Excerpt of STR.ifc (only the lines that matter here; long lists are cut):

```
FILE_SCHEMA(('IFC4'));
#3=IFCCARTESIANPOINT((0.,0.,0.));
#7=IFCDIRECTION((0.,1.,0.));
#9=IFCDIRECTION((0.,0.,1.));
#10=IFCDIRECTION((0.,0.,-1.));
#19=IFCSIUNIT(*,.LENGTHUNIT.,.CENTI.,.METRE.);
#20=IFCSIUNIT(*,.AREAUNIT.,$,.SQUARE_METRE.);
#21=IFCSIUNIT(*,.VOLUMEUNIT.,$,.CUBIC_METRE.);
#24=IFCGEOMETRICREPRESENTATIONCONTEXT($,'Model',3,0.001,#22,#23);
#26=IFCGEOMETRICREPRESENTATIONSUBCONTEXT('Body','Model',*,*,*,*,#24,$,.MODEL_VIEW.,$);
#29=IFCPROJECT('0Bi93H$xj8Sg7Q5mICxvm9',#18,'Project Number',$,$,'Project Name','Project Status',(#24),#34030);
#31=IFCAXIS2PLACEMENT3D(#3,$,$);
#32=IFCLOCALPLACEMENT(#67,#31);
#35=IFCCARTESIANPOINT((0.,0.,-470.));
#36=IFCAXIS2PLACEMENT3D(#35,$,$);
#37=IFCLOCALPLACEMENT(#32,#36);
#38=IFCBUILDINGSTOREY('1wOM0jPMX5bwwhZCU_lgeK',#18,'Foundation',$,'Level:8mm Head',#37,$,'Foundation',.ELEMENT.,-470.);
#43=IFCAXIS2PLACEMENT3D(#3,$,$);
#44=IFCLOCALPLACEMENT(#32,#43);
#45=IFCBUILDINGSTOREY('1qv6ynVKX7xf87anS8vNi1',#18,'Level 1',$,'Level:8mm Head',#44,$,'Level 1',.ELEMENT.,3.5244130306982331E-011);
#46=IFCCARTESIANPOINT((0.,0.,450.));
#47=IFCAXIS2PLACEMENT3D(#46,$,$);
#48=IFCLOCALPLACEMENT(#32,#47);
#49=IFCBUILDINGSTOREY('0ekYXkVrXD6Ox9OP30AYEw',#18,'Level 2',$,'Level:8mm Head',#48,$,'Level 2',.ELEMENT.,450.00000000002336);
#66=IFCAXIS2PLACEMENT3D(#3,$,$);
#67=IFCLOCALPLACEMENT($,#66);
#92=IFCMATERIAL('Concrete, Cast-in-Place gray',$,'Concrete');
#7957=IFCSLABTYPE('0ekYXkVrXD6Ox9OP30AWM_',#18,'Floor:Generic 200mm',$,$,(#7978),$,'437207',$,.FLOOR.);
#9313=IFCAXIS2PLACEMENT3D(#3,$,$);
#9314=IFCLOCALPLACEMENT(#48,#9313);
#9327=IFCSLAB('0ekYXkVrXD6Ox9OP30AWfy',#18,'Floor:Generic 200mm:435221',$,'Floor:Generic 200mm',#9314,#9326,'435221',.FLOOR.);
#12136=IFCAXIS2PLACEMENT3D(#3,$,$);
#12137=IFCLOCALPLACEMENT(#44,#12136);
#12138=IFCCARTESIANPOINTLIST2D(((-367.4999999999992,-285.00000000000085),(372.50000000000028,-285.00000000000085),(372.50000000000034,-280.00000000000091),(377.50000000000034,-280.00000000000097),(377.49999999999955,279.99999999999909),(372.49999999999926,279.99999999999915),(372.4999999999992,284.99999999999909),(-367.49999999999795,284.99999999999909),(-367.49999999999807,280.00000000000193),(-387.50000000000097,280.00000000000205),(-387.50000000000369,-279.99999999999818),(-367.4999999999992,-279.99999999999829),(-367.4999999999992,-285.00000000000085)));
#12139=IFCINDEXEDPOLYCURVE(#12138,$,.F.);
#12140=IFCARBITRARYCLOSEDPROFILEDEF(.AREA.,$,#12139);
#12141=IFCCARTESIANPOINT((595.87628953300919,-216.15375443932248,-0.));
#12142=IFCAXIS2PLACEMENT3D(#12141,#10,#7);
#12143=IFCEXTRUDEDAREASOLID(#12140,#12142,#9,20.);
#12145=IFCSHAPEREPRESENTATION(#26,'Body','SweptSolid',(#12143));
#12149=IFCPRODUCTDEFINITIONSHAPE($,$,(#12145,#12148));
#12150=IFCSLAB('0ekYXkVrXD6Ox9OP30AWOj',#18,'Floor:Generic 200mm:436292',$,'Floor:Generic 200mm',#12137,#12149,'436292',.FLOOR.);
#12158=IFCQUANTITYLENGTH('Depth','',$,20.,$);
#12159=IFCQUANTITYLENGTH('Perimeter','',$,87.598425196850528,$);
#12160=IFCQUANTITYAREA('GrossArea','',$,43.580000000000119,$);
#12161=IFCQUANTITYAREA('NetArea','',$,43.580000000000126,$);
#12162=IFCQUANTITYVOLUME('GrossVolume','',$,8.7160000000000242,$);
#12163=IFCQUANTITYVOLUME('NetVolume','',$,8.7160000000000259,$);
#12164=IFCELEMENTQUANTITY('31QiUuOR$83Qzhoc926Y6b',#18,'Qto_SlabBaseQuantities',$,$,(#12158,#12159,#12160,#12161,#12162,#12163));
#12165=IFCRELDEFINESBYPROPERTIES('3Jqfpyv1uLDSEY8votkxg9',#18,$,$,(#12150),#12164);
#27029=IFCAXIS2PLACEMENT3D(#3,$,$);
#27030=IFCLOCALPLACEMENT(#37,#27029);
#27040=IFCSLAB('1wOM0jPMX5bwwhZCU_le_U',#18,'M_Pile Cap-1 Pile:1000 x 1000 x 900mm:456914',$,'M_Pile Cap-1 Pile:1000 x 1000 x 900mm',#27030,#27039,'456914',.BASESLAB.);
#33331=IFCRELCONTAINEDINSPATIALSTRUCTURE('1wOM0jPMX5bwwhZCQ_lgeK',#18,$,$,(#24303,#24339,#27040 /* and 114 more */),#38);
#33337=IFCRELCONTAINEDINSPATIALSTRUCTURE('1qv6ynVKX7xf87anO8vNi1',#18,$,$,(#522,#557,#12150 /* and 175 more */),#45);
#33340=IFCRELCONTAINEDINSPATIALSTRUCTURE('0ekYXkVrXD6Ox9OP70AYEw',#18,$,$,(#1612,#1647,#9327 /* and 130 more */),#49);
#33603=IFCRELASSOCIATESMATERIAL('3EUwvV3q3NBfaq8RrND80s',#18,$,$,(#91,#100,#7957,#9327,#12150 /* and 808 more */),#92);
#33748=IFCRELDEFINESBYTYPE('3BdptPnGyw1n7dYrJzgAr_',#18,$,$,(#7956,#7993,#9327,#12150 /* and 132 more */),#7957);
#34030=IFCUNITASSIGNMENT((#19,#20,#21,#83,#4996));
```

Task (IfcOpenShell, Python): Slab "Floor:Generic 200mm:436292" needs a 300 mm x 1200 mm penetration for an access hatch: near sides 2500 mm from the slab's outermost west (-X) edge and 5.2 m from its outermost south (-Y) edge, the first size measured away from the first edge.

```python
import numpy as np
import ifcopenshell
import ifcopenshell.api.feature
import ifcopenshell.api.geometry
import ifcopenshell.api.pset
import ifcopenshell.api.root
import ifcopenshell.geom
import ifcopenshell.util.element
import ifcopenshell.util.placement
import ifcopenshell.util.representation
import ifcopenshell.util.shape
import ifcopenshell.util.unit

model = ifcopenshell.open("STR.ifc")
unit_scale = ifcopenshell.util.unit.calculate_unit_scale(model)
area_scale = ifcopenshell.util.unit.calculate_unit_scale(model, "AREAUNIT")
volume_scale = ifcopenshell.util.unit.calculate_unit_scale(model, "VOLUMEUNIT")
settings = ifcopenshell.geom.settings()


def volume(element):
    """Net volume in cubic metres, openings subtracted."""
    shape = ifcopenshell.geom.create_shape(settings, element)
    return ifcopenshell.util.shape.get_volume(shape.geometry)


slab = model.by_guid("0ekYXkVrXD6Ox9OP30AWOj")
before = volume(slab)

# Extent in the slab's own axes, in metres. The edges named are its -X and -Y sides.
slab_shape = ifcopenshell.geom.create_shape(settings, slab)
vertices = ifcopenshell.util.shape.get_vertices(slab_shape.geometry)
x_min, y_min, bottom = vertices.min(axis=0)
top = vertices[:, 2].max()

opening = ifcopenshell.api.root.create_entity(model, ifc_class="IfcOpeningElement", name="Access hatch opening", predefined_type="OPENING")
context = ifcopenshell.util.representation.get_context(model, "Model", "Body", "MODEL_VIEW")
width, depth = 0.3, 1.2
outline = [(0.0, 0.0), (width, 0.0), (width, depth), (0.0, depth), (0.0, 0.0)]
# Overshoot both faces by 50 mm so the cut is clean.
shape = ifcopenshell.api.geometry.add_slab_representation(
    model, context=context, depth=top - bottom + 0.1, polyline=outline
)
ifcopenshell.api.geometry.assign_representation(model, product=opening, representation=shape)

matrix = ifcopenshell.util.placement.get_local_placement(slab.ObjectPlacement)
matrix[:, 3] = matrix @ np.append(np.array([x_min + 2.5, y_min + 5.2, bottom - 0.05]) / unit_scale, 1.0)
ifcopenshell.api.geometry.edit_object_placement(model, product=opening, matrix=matrix, is_si=False)
ifcopenshell.api.feature.add_feature(model, feature=opening, element=slab)

after = volume(slab)

# Update the slab's stored quantities.
qto = model.by_id(ifcopenshell.util.element.get_pset(slab, "Qto_SlabBaseQuantities", should_inherit=False)["id"])
ifcopenshell.api.pset.edit_qto(model, qto=qto, properties={
    "NetArea": after / (top - bottom) / area_scale,
    "NetVolume": after / volume_scale,
})

print(f"slab volume {before:.3f} -> {after:.3f} m3")

model.write("STR_v2.ifc")
```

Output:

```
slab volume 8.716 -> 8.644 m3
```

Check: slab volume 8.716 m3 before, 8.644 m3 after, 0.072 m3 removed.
